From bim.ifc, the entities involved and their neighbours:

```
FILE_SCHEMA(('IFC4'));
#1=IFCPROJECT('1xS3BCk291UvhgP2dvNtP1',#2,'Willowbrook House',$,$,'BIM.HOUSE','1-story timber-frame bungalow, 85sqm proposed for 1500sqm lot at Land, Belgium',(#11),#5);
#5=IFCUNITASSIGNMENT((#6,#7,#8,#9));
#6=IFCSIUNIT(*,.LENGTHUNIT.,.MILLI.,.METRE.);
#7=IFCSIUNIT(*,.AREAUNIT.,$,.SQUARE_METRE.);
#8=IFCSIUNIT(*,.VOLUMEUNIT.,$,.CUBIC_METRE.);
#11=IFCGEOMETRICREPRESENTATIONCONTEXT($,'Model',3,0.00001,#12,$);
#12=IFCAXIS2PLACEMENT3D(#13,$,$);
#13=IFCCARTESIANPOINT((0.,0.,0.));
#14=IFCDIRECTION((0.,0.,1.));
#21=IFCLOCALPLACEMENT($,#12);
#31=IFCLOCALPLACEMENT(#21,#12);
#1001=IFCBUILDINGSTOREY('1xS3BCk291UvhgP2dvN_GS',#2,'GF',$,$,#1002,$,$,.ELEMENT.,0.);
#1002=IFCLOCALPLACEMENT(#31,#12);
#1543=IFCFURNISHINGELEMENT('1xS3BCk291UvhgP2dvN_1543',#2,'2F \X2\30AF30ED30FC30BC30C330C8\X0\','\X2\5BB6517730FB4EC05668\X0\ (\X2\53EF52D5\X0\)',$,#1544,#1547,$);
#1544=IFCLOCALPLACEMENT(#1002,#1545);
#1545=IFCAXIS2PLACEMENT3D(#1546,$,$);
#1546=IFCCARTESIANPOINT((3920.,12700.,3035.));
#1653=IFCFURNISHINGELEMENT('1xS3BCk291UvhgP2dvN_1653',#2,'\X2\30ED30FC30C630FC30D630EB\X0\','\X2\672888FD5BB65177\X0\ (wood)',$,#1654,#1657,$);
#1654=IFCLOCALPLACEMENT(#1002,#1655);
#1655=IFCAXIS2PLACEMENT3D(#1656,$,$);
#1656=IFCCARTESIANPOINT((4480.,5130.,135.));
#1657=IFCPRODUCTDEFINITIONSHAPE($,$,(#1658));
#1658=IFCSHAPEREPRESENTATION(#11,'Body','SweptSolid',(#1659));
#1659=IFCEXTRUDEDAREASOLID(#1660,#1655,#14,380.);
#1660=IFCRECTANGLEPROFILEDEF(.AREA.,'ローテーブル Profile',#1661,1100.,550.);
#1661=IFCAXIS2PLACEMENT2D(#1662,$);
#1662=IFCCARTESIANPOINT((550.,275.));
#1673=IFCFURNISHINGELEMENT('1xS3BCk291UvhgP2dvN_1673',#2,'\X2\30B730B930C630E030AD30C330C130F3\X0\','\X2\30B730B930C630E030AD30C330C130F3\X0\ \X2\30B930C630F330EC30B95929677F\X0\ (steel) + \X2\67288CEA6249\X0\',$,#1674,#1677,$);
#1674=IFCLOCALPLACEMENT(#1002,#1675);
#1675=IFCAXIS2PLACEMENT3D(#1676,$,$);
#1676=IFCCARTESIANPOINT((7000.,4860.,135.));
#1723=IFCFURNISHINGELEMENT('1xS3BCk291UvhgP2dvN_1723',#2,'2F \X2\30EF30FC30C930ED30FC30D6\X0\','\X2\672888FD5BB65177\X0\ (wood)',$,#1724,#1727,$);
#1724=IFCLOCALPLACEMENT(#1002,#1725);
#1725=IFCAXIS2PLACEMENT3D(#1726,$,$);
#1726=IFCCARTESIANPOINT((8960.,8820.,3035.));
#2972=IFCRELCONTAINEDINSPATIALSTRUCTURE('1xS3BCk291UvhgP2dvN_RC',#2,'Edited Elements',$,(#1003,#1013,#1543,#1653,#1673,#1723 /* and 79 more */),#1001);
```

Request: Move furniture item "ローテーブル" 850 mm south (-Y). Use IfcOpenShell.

```python
import ifcopenshell
import ifcopenshell.api.geometry
import ifcopenshell.util.placement
import ifcopenshell.util.unit

model = ifcopenshell.open("bim.ifc")
unit_scale = ifcopenshell.util.unit.calculate_unit_scale(model)

item = model.by_id(1653)
matrix = ifcopenshell.util.placement.get_local_placement(item.ObjectPlacement)
matrix[1, 3] -= 0.85 / unit_scale
ifcopenshell.api.geometry.edit_object_placement(model, product=item, matrix=matrix, is_si=False)

print(ifcopenshell.util.placement.get_local_placement(item.ObjectPlacement).round(3) + 0.0)

model.write("bim_edited.ifc")
```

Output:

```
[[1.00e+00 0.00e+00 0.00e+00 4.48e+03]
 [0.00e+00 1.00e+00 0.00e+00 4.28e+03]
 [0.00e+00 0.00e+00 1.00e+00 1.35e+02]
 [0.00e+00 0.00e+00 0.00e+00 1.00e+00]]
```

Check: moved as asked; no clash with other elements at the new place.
